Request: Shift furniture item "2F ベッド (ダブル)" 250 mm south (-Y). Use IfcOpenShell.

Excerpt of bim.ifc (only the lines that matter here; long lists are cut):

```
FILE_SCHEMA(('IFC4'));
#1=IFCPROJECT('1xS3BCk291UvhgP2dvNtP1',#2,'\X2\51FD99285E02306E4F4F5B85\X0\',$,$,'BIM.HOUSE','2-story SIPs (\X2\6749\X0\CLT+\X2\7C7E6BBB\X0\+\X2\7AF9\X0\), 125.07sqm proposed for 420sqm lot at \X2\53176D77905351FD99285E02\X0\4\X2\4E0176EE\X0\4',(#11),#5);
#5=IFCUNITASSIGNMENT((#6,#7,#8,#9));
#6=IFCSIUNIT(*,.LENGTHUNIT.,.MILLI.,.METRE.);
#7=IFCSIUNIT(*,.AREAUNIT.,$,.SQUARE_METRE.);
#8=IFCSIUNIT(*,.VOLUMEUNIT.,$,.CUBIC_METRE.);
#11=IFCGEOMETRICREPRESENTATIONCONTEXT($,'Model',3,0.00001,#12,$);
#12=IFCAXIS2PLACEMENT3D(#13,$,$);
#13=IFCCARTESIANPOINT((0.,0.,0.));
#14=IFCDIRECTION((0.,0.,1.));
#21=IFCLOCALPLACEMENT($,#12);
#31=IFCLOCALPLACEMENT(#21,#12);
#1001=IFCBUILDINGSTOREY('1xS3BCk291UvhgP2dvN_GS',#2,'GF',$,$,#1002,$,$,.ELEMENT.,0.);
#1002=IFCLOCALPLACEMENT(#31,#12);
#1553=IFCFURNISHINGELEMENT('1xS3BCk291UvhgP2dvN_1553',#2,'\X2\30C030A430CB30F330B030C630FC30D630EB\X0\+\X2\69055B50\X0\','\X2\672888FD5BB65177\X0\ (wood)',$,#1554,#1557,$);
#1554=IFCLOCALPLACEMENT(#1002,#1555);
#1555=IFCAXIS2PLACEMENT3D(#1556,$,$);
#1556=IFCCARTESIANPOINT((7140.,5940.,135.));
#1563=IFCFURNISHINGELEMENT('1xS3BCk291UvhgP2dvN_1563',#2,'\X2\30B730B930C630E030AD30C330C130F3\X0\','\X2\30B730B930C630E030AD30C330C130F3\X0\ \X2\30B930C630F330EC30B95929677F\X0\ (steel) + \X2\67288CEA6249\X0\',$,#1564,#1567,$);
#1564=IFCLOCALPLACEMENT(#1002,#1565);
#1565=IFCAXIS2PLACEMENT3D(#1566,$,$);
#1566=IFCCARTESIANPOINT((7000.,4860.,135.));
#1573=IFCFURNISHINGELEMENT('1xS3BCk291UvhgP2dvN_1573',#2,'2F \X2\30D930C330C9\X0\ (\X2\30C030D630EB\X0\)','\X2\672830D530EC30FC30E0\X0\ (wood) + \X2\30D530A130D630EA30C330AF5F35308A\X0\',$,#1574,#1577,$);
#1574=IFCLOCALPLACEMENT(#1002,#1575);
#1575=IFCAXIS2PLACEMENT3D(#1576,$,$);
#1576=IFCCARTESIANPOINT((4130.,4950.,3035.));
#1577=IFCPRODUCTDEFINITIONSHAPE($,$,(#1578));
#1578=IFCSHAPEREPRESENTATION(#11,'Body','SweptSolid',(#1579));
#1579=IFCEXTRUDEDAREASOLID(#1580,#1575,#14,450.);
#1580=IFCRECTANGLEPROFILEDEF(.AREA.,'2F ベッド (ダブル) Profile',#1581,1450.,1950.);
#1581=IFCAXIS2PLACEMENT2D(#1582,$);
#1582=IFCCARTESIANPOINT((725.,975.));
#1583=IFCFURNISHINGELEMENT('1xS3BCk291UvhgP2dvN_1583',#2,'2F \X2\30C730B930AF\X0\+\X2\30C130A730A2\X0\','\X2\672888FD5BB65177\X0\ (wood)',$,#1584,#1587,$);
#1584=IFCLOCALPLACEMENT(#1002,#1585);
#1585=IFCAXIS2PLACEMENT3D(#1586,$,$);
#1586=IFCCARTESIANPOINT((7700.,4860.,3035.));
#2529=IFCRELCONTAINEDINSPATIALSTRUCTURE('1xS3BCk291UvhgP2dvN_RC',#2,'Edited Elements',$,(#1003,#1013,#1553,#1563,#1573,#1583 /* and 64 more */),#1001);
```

```python
import ifcopenshell
import ifcopenshell.api.geometry
import ifcopenshell.util.placement

model = ifcopenshell.open("bim.ifc")

item = model.by_id(1573)
matrix = ifcopenshell.util.placement.get_local_placement(item.ObjectPlacement)
matrix[1, 3] -= 250.0
ifcopenshell.api.geometry.edit_object_placement(model, product=item, matrix=matrix, is_si=False)

print(ifcopenshell.util.placement.get_local_placement(item.ObjectPlacement).round(3) + 0.0)

model.write("bim_edited.ifc")
```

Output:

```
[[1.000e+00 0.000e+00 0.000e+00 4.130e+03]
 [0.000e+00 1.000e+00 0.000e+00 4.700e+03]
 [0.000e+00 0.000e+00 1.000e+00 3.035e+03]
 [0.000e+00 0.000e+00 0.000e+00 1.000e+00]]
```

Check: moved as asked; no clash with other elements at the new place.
